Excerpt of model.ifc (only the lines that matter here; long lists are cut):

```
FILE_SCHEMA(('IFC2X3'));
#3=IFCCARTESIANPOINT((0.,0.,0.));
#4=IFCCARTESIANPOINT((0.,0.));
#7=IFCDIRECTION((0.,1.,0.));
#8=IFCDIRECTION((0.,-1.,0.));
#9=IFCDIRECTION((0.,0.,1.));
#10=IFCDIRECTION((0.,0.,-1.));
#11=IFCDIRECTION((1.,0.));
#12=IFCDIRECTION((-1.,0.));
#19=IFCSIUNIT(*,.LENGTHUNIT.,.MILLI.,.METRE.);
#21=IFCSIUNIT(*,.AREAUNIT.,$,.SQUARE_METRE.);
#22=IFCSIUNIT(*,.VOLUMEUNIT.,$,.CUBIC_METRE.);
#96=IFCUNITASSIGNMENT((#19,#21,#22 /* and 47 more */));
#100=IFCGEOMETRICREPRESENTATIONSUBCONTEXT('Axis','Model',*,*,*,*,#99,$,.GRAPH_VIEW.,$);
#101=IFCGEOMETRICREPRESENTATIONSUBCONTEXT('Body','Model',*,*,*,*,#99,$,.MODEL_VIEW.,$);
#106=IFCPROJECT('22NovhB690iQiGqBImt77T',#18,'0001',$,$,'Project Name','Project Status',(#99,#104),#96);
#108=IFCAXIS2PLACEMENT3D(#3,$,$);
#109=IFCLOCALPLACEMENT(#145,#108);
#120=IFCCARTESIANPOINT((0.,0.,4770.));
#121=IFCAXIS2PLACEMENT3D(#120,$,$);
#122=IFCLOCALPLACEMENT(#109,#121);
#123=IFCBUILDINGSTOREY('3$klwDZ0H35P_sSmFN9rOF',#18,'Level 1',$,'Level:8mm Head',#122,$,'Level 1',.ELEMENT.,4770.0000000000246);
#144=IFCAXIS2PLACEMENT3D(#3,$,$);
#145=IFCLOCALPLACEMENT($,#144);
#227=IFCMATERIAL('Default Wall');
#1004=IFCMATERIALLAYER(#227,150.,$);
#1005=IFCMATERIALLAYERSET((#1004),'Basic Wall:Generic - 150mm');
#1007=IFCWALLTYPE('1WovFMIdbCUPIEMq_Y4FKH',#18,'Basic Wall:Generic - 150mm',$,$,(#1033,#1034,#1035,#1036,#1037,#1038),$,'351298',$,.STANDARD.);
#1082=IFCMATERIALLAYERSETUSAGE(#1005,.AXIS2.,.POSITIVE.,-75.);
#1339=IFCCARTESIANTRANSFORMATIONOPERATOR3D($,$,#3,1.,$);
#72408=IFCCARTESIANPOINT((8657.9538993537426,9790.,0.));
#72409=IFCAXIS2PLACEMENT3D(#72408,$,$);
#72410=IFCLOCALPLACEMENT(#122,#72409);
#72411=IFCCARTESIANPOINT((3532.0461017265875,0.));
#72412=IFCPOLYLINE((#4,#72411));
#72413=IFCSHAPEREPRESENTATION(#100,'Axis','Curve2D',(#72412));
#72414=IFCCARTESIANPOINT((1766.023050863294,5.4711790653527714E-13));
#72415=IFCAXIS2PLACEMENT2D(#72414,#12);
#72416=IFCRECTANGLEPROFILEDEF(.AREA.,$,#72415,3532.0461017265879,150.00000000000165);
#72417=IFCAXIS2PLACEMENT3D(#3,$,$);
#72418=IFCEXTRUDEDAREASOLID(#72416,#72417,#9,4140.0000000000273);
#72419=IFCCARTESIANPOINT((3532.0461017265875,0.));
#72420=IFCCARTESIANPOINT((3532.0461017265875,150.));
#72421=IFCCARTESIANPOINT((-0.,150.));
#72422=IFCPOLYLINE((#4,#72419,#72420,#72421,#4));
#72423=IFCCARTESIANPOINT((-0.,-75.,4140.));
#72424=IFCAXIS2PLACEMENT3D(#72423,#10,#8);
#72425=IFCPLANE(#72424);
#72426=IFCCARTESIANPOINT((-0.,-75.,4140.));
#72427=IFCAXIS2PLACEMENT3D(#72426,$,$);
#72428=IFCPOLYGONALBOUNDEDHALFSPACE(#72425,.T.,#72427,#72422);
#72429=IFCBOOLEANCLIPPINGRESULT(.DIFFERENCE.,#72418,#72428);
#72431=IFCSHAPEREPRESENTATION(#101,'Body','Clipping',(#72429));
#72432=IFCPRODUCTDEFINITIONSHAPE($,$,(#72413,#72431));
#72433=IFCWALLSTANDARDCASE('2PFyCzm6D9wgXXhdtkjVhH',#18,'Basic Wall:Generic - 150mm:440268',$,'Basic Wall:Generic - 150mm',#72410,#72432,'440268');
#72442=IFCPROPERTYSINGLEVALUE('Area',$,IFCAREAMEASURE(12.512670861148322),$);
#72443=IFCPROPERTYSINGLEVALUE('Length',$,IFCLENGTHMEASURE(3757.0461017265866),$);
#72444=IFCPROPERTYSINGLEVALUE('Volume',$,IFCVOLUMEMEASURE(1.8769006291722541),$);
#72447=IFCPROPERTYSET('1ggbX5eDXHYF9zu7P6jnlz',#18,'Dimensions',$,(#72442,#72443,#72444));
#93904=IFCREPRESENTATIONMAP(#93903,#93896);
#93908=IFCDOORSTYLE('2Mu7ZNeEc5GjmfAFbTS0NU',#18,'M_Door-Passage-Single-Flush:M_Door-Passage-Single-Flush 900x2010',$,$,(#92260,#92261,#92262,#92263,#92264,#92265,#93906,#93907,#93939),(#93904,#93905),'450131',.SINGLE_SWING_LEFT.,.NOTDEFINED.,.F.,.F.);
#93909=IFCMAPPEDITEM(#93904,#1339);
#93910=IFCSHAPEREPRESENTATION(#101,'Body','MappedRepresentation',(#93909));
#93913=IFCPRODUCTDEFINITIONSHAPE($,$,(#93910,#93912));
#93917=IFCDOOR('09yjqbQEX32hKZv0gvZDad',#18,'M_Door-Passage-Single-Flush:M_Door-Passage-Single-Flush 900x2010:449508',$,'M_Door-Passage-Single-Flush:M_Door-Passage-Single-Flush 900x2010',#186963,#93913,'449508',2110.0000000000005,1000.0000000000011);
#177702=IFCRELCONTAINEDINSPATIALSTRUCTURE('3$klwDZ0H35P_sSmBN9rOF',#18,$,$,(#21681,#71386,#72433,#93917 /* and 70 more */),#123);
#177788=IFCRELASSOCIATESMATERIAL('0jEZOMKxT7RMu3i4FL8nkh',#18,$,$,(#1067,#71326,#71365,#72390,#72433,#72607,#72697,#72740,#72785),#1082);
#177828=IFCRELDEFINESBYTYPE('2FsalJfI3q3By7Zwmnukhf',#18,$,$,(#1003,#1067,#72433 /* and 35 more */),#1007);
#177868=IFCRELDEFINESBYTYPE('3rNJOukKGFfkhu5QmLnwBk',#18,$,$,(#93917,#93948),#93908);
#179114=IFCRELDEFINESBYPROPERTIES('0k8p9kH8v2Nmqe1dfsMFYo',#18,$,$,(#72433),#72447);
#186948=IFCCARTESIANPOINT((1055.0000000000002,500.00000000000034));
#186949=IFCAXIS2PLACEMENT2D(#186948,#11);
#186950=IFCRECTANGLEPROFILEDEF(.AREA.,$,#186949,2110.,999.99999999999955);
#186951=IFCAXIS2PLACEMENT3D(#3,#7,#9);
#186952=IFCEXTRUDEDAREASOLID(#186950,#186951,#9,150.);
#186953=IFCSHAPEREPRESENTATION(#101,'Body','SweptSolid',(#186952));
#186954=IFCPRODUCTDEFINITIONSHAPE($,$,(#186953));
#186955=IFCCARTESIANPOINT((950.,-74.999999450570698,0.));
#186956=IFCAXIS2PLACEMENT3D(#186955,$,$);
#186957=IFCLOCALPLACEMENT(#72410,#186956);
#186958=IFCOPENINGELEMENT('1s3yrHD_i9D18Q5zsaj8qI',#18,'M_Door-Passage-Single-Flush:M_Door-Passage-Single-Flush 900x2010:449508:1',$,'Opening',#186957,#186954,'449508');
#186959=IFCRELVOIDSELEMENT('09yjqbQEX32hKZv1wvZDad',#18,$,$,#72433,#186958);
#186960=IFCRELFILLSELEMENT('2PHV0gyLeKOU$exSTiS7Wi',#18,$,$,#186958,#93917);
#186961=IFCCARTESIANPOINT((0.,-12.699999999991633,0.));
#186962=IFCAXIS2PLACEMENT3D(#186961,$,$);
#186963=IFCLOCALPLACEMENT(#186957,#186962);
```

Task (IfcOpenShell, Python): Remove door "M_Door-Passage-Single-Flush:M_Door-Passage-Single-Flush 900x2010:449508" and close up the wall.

```python
import ifcopenshell
import ifcopenshell.api.feature
import ifcopenshell.api.pset
import ifcopenshell.api.root
import ifcopenshell.geom
import ifcopenshell.util.element
import ifcopenshell.util.shape
import ifcopenshell.util.unit

model = ifcopenshell.open("model.ifc")
area_scale = ifcopenshell.util.unit.calculate_unit_scale(model, "AREAUNIT")
volume_scale = ifcopenshell.util.unit.calculate_unit_scale(model, "VOLUMEUNIT")
settings = ifcopenshell.geom.settings()


def volume(element):
    """Net volume in cubic metres, openings subtracted."""
    shape = ifcopenshell.geom.create_shape(settings, element)
    return ifcopenshell.util.shape.get_volume(shape.geometry)


door = model.by_guid("09yjqbQEX32hKZv0gvZDad")
opening = door.FillsVoids[0].RelatingOpeningElement
wall = opening.VoidsElements[0].RelatingBuildingElement
before = volume(wall)

ifcopenshell.api.root.remove_product(model, product=door)
ifcopenshell.api.feature.remove_feature(model, feature=opening)

after = volume(wall)
thickness = 0.15  # wall thickness in metres

# Update the wall's stored quantities.
pset = model.by_id(ifcopenshell.util.element.get_pset(wall, "Dimensions", should_inherit=False)["id"])
ifcopenshell.api.pset.edit_pset(model, pset=pset, properties={
    "Area": model.create_entity("IfcAreaMeasure", after / thickness / area_scale),
    "Volume": model.create_entity("IfcVolumeMeasure", after / volume_scale),
})

print(f"wall volume {before:.3f} -> {after:.3f} m3")

model.write("model_updated.ifc")
```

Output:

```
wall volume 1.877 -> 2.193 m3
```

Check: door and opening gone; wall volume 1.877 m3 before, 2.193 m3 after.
